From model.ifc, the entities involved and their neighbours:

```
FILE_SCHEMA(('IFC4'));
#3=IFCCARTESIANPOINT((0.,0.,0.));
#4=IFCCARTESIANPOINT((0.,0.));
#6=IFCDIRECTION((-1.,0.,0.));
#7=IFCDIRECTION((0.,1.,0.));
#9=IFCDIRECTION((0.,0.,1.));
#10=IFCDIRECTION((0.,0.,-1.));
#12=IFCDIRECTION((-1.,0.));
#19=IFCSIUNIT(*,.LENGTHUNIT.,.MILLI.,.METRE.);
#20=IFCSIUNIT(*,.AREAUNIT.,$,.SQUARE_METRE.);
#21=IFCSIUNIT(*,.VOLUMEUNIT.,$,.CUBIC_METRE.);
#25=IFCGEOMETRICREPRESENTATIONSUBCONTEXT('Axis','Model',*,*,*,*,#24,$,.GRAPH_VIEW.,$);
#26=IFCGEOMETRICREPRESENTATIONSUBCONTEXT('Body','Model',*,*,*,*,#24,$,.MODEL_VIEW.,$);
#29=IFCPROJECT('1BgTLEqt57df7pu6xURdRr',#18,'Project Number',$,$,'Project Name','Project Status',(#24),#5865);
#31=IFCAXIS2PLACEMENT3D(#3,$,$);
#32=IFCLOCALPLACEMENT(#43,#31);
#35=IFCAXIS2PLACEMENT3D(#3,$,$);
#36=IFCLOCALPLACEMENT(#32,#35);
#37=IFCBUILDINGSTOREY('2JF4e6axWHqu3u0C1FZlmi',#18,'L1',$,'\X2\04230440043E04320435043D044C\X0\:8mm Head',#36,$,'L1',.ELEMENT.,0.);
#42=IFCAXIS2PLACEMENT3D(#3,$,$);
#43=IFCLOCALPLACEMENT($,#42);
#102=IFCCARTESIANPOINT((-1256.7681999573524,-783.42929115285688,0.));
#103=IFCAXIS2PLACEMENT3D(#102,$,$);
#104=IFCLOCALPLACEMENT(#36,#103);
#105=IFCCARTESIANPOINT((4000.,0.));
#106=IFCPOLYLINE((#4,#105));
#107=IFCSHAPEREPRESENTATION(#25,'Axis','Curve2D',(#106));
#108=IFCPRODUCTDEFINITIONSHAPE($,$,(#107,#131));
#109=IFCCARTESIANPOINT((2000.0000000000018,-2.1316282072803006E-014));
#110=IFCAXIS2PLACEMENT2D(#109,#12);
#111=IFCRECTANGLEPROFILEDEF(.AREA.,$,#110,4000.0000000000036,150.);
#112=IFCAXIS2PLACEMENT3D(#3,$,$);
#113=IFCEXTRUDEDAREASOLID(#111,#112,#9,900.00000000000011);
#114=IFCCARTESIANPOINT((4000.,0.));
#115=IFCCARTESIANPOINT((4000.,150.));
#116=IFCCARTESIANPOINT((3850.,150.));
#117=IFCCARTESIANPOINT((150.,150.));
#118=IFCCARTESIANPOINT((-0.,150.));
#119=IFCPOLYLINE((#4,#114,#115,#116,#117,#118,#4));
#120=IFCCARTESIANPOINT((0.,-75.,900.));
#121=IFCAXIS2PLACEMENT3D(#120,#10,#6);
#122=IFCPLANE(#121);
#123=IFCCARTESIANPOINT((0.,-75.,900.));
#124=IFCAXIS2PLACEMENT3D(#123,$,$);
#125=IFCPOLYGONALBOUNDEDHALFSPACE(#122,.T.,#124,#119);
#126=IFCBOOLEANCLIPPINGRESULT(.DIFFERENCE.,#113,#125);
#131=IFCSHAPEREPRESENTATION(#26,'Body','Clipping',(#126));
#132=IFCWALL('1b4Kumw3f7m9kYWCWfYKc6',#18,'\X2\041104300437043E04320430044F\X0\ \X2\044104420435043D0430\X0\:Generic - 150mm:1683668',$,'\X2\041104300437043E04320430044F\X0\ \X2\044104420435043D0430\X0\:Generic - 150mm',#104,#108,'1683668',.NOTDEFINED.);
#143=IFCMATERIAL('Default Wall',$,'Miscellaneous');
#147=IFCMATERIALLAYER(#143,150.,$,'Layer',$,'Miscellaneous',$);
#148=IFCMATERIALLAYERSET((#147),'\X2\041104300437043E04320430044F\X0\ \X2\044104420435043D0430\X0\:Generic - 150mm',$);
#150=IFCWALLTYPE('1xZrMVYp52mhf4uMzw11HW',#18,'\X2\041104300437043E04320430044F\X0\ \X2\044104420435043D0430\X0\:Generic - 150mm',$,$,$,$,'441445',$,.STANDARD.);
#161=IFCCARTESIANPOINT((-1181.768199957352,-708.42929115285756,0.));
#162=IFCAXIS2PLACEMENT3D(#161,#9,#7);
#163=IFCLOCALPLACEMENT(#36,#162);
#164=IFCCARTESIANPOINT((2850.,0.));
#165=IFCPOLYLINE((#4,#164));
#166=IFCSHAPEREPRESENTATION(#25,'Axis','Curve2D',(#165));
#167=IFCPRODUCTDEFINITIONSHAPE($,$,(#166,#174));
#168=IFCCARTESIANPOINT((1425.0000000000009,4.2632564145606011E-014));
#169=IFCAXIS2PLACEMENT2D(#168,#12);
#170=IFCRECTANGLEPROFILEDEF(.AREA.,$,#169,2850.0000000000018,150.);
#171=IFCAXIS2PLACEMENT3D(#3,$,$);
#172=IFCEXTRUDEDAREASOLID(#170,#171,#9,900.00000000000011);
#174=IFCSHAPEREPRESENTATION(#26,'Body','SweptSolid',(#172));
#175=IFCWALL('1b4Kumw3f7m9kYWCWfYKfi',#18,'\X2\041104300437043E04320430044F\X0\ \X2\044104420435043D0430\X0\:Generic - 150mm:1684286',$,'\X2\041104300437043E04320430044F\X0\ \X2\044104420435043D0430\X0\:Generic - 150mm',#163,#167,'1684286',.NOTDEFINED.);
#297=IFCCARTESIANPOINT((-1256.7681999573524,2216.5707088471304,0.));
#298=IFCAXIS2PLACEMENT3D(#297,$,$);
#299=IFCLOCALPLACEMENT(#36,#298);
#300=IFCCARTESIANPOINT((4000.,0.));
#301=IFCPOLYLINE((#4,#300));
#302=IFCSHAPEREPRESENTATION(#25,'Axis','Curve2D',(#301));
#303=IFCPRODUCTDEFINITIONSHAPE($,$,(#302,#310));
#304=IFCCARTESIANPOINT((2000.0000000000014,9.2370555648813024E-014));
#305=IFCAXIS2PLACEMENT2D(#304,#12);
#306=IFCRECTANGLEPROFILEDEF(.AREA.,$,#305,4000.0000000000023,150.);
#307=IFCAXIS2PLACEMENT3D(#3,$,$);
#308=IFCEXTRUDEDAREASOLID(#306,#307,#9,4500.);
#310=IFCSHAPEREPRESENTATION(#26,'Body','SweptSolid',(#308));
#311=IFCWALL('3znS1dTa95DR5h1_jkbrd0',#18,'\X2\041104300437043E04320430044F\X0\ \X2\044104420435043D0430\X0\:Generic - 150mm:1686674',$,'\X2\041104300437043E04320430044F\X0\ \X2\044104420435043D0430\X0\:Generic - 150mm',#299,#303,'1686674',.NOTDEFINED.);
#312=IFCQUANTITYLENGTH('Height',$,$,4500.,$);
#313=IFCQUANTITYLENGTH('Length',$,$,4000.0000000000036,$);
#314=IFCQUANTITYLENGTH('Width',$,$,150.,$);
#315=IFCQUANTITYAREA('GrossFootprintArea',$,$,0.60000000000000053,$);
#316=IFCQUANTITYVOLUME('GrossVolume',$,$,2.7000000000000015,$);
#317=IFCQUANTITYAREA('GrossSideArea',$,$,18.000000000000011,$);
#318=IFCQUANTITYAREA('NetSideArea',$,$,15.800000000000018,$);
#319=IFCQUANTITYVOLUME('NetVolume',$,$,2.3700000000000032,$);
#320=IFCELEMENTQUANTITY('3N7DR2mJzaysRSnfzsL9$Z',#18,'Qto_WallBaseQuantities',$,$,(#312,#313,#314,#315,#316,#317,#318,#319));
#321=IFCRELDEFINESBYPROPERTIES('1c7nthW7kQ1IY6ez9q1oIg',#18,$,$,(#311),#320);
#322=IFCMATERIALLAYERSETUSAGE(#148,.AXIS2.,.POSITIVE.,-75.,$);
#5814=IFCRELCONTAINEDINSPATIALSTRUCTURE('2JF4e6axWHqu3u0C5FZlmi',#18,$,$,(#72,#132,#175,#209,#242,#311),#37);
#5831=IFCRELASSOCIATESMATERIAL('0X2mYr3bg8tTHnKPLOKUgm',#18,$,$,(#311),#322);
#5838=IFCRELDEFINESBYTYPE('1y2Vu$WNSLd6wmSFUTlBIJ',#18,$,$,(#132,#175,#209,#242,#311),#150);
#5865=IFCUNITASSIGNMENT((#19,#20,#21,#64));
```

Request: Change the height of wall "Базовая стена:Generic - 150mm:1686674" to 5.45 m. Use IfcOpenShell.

```python
import ifcopenshell
import ifcopenshell.api.pset
import ifcopenshell.geom
import ifcopenshell.util.element
import ifcopenshell.util.representation
import ifcopenshell.util.shape
import ifcopenshell.util.unit

model = ifcopenshell.open("model.ifc")
unit_scale = ifcopenshell.util.unit.calculate_unit_scale(model)
area_scale = ifcopenshell.util.unit.calculate_unit_scale(model, "AREAUNIT")
volume_scale = ifcopenshell.util.unit.calculate_unit_scale(model, "VOLUMEUNIT")
settings = ifcopenshell.geom.settings()


def volume(element):
    """Net volume in cubic metres, openings subtracted."""
    shape = ifcopenshell.geom.create_shape(settings, element)
    return ifcopenshell.util.shape.get_volume(shape.geometry)


wall = model.by_guid("3znS1dTa95DR5h1_jkbrd0")
before = volume(wall)

body = ifcopenshell.util.representation.get_representation(wall, "Model", "Body")
solid = body.Items[0]
old_height = solid.Depth
solid.Depth = 5.45 / unit_scale
after = volume(wall)
thickness = 0.15  # wall thickness in metres

# Update the stored height, areas and volumes.
qto = model.by_id(ifcopenshell.util.element.get_pset(wall, "Qto_WallBaseQuantities", should_inherit=False)["id"])
ifcopenshell.api.pset.edit_qto(model, qto=qto, properties={
    "Height": solid.Depth,
    "GrossVolume": ifcopenshell.util.element.get_pset(wall, "Qto_WallBaseQuantities", "GrossVolume") * solid.Depth / old_height,
    "GrossSideArea": ifcopenshell.util.element.get_pset(wall, "Qto_WallBaseQuantities", "GrossSideArea") * solid.Depth / old_height,
    "NetSideArea": after / thickness / area_scale,
    "NetVolume": after / volume_scale,
})

print(f"height {old_height:g} -> {solid.Depth:g}, volume {before:.3f} -> {after:.3f} m3")

model.write("model_updated.ifc")
```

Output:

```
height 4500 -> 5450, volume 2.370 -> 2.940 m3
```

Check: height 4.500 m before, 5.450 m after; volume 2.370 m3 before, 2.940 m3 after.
